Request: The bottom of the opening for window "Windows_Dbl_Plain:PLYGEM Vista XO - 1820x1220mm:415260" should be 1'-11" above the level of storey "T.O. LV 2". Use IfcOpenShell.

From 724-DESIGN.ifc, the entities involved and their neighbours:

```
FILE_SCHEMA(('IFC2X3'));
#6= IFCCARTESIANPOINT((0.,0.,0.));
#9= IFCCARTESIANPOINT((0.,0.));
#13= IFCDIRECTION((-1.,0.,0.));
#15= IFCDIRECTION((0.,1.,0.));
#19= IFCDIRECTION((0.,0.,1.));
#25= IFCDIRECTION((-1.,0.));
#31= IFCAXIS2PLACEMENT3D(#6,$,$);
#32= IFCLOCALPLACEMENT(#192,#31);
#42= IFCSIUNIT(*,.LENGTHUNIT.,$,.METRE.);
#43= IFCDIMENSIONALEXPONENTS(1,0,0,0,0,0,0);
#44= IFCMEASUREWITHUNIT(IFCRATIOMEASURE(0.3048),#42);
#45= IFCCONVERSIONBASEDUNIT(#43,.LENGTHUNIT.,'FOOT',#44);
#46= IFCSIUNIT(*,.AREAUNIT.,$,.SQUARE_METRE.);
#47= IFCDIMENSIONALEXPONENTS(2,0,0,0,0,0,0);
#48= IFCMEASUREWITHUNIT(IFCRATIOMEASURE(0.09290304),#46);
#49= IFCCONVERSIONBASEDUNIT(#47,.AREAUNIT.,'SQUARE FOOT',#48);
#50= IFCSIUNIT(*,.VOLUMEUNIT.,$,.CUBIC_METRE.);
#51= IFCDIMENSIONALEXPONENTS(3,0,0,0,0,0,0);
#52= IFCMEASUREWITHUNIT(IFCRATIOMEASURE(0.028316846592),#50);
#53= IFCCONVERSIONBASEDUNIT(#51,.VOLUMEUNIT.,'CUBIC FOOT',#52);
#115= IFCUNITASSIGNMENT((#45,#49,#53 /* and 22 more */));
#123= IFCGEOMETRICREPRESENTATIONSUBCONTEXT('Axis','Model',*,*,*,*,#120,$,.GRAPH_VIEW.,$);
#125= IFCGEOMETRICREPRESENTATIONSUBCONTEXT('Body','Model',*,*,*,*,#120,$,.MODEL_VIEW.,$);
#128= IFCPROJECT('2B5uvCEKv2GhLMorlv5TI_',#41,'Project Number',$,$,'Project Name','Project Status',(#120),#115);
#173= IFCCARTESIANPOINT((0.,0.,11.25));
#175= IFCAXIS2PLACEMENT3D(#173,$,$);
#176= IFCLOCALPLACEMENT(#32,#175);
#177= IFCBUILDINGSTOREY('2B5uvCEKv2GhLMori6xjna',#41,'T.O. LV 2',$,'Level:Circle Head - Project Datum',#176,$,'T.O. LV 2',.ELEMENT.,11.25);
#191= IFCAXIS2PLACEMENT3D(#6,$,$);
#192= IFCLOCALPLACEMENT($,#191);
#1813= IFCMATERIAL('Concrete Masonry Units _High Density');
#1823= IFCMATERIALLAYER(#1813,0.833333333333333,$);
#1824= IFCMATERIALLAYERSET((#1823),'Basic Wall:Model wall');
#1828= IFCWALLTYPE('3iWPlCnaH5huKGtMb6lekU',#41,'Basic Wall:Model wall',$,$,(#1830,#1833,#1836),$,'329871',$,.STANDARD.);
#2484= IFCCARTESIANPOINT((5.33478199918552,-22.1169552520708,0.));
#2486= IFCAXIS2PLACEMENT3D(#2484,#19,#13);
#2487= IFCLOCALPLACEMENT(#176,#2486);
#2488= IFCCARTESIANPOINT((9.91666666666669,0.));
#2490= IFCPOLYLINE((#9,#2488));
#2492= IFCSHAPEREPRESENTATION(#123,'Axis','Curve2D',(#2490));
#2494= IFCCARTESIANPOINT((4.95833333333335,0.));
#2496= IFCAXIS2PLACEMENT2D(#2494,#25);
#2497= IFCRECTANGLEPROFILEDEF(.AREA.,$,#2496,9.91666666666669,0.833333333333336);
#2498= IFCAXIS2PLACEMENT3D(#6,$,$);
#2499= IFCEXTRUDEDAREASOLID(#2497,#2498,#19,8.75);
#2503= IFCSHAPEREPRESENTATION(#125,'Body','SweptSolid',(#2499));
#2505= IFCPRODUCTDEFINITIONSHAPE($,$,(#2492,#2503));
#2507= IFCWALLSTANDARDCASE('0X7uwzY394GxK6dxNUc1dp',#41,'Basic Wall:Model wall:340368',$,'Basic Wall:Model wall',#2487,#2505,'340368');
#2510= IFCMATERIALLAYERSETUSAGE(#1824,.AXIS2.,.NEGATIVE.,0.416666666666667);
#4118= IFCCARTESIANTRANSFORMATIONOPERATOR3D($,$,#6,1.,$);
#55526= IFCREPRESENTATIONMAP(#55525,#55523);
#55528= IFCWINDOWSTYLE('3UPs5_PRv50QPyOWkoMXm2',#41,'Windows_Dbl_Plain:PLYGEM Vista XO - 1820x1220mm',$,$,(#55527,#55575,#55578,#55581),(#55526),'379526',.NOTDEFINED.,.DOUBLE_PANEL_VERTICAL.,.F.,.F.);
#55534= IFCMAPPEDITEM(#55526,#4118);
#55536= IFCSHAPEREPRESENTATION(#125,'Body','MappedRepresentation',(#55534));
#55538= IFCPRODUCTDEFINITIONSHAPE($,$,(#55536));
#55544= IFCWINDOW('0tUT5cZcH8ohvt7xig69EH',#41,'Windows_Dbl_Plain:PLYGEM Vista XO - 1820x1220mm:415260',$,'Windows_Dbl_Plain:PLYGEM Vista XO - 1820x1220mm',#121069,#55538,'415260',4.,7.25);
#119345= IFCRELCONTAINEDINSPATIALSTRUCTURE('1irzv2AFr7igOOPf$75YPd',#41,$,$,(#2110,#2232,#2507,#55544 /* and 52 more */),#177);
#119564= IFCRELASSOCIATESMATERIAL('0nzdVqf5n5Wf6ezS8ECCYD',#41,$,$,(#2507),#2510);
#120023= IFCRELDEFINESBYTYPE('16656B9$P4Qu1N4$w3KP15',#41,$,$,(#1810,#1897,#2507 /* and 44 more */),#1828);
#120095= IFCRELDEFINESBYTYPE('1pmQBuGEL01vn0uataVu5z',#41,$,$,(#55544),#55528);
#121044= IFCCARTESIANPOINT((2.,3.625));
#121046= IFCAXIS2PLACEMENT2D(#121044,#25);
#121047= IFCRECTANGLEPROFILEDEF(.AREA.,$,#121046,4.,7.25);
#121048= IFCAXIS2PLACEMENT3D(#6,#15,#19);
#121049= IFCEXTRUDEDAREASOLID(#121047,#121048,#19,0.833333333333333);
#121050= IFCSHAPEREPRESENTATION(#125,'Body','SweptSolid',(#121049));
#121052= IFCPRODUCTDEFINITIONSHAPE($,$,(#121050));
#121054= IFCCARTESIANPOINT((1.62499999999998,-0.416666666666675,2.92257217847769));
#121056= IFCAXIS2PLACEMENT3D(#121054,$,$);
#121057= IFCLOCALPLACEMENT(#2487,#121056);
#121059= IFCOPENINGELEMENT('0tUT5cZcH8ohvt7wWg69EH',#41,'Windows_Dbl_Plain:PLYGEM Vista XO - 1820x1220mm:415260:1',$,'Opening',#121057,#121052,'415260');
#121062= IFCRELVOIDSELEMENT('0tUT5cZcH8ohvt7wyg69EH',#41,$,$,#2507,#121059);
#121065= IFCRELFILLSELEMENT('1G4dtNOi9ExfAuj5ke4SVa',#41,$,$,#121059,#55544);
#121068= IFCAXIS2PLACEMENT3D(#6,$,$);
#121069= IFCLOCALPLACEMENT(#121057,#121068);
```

```python
import numpy as np
import ifcopenshell
import ifcopenshell.api.geometry
import ifcopenshell.geom
import ifcopenshell.util.element
import ifcopenshell.util.placement
import ifcopenshell.util.shape
import ifcopenshell.util.unit

model = ifcopenshell.open("724-DESIGN.ifc")
unit_scale = ifcopenshell.util.unit.calculate_unit_scale(model)

window = model.by_guid("0tUT5cZcH8ohvt7xig69EH")
opening = window.FillsVoids[0].RelatingOpeningElement
storey = ifcopenshell.util.element.get_container(window, ifc_class="IfcBuildingStorey")
level = ifcopenshell.util.placement.get_local_placement(storey.ObjectPlacement)[2, 3]

# The opening's origin need not be at the sill, so measure its lowest point.
shape = ifcopenshell.geom.create_shape(ifcopenshell.geom.settings(), opening)
bottom = ifcopenshell.util.shape.get_shape_bottom_elevation(shape, shape.geometry) / unit_scale
dz = level + 23 * 0.0254 / unit_scale - bottom

shift = np.array([0.0, 0.0, dz])
# The window is placed relative to its opening, so it follows when the opening moves.
matrix = ifcopenshell.util.placement.get_local_placement(opening.ObjectPlacement)
matrix[:3, 3] += shift
ifcopenshell.api.geometry.edit_object_placement(
    model, product=opening, matrix=matrix, is_si=False, should_transform_children=True
)

print(f"moved by {dz * unit_scale:+.3f} m")

model.write("724-DESIGN_updated.ifc")
```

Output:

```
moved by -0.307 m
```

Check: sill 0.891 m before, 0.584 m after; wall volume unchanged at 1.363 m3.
